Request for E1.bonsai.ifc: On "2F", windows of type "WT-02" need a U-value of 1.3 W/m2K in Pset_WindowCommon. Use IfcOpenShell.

First a look at what the model holds.

```python
import ifcopenshell
import ifcopenshell.util.element

model = ifcopenshell.open("E1.bonsai.ifc")
print(model.schema)
storey = next(s for s in model.by_type("IfcBuildingStorey") if s.Name == "2F")
windows = [e for e in ifcopenshell.util.element.get_decomposition(storey) if e.is_a("IfcWindow")]
seen = {}
for e in windows:
    element_type = ifcopenshell.util.element.get_type(e)
    key = (element_type.Name if element_type != e and element_type else None, ifcopenshell.util.element.get_pset(e, "Pset_WindowCommon", "ThermalTransmittance"))
    seen[key] = seen.get(key, 0) + 1
for (name, value), count in sorted(seen.items(), key=str):
    print(count, "x", name, "|", value)
```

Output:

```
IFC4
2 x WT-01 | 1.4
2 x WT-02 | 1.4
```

```python
import ifcopenshell
import ifcopenshell.api.pset
import ifcopenshell.util.element

model = ifcopenshell.open("E1.bonsai.ifc")

storey = next(s for s in model.by_type("IfcBuildingStorey") if s.Name == "2F")
windows = [e for e in ifcopenshell.util.element.get_decomposition(storey) if e.is_a("IfcWindow")]

count = 0
for e in windows:
    element_type = ifcopenshell.util.element.get_type(e)
    if element_type in (None, e) or element_type.Name != "WT-02":
        continue
    # add_pset returns the element's existing set when there is one.
    pset = ifcopenshell.api.pset.add_pset(model, product=e, name="Pset_WindowCommon")
    ifcopenshell.api.pset.edit_pset(model, pset=pset, properties={"ThermalTransmittance": 1.3})
    count += 1

print(count, "windows updated")

model.write("E1.bonsai_rev.ifc")
```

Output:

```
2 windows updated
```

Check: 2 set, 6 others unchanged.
